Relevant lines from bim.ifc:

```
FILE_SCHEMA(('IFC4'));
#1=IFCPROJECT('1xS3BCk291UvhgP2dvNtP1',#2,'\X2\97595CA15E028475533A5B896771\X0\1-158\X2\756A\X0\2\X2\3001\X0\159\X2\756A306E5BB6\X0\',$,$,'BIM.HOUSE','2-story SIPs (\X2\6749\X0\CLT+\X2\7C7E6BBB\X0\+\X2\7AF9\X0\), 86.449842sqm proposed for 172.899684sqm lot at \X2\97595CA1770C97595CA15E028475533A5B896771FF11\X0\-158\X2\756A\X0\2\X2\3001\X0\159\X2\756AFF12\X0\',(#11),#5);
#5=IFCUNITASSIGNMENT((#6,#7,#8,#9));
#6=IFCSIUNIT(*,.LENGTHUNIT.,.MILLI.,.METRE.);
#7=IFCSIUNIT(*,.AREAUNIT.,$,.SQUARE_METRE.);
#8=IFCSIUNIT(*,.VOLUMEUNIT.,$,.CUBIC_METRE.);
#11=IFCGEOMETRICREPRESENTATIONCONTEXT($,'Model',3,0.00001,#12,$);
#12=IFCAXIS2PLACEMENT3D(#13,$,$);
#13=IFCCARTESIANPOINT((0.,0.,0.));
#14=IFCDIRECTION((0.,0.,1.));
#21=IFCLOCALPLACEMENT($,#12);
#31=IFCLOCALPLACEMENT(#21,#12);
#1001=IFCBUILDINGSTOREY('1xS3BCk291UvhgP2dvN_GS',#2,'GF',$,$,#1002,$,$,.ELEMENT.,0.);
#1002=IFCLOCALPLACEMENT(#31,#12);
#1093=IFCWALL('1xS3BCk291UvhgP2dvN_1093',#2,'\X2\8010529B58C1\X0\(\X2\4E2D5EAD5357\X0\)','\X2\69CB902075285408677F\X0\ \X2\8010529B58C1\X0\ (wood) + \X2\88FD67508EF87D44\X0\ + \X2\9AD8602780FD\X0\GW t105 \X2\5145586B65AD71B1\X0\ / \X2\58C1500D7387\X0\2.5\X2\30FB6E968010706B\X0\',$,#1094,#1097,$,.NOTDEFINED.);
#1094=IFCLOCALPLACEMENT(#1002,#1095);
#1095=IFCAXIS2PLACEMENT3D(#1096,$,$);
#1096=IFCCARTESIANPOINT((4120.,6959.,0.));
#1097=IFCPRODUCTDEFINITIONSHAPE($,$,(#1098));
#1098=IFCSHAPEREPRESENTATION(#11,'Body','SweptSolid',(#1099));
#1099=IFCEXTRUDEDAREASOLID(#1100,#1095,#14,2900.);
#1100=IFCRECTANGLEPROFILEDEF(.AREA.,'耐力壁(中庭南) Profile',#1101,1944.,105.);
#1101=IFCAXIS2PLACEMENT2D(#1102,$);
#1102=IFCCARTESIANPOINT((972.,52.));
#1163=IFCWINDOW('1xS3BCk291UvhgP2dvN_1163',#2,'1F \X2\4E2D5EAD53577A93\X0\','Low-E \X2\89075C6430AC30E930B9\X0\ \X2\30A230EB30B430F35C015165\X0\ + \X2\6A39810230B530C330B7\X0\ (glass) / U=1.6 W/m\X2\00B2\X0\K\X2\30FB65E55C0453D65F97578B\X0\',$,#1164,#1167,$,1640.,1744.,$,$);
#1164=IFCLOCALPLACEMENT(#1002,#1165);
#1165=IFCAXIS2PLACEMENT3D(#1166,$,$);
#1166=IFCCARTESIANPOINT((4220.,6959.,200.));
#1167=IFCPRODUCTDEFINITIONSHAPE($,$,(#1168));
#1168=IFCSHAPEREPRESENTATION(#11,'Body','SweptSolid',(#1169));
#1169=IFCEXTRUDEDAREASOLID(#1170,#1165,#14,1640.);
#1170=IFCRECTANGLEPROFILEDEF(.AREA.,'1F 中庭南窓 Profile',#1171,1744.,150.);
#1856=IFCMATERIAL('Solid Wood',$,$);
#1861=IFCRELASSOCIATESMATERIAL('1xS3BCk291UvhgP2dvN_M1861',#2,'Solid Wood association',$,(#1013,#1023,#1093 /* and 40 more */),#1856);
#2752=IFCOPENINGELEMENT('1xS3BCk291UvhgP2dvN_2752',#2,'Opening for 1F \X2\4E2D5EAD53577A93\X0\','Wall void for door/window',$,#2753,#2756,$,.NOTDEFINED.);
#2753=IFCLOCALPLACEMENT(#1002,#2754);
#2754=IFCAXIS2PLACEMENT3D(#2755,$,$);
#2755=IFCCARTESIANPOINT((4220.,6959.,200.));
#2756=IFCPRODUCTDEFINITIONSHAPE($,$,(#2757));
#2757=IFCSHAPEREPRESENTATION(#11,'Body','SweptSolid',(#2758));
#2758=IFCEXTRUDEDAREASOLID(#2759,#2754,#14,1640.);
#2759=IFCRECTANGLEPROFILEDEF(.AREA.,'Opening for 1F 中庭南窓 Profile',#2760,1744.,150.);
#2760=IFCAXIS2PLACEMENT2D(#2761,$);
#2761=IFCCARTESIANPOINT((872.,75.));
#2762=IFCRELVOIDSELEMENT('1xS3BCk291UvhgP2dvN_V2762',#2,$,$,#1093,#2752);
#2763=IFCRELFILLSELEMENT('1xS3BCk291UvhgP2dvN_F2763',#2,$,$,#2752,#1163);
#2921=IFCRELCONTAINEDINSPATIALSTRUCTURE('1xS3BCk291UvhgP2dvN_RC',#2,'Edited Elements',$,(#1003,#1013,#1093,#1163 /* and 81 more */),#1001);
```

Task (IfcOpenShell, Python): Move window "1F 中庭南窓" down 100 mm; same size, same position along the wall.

```python
import numpy as np
import ifcopenshell
import ifcopenshell.api.geometry
import ifcopenshell.util.placement
import ifcopenshell.util.unit

model = ifcopenshell.open("bim.ifc")
unit_scale = ifcopenshell.util.unit.calculate_unit_scale(model)

window = model.by_guid("1xS3BCk291UvhgP2dvN_1163")
opening = window.FillsVoids[0].RelatingOpeningElement
dz = -100.0

shift = np.array([0.0, 0.0, dz])
# The window is not placed relative to its opening, so move both.
for product in (opening, window):
    matrix = ifcopenshell.util.placement.get_local_placement(product.ObjectPlacement)
    matrix[:3, 3] += shift
    ifcopenshell.api.geometry.edit_object_placement(model, product=product, matrix=matrix, is_si=False)

print(f"moved by {dz * unit_scale:+.3f} m")

model.write("bim_updated.ifc")
```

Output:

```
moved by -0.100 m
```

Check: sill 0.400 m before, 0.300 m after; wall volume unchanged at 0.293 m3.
